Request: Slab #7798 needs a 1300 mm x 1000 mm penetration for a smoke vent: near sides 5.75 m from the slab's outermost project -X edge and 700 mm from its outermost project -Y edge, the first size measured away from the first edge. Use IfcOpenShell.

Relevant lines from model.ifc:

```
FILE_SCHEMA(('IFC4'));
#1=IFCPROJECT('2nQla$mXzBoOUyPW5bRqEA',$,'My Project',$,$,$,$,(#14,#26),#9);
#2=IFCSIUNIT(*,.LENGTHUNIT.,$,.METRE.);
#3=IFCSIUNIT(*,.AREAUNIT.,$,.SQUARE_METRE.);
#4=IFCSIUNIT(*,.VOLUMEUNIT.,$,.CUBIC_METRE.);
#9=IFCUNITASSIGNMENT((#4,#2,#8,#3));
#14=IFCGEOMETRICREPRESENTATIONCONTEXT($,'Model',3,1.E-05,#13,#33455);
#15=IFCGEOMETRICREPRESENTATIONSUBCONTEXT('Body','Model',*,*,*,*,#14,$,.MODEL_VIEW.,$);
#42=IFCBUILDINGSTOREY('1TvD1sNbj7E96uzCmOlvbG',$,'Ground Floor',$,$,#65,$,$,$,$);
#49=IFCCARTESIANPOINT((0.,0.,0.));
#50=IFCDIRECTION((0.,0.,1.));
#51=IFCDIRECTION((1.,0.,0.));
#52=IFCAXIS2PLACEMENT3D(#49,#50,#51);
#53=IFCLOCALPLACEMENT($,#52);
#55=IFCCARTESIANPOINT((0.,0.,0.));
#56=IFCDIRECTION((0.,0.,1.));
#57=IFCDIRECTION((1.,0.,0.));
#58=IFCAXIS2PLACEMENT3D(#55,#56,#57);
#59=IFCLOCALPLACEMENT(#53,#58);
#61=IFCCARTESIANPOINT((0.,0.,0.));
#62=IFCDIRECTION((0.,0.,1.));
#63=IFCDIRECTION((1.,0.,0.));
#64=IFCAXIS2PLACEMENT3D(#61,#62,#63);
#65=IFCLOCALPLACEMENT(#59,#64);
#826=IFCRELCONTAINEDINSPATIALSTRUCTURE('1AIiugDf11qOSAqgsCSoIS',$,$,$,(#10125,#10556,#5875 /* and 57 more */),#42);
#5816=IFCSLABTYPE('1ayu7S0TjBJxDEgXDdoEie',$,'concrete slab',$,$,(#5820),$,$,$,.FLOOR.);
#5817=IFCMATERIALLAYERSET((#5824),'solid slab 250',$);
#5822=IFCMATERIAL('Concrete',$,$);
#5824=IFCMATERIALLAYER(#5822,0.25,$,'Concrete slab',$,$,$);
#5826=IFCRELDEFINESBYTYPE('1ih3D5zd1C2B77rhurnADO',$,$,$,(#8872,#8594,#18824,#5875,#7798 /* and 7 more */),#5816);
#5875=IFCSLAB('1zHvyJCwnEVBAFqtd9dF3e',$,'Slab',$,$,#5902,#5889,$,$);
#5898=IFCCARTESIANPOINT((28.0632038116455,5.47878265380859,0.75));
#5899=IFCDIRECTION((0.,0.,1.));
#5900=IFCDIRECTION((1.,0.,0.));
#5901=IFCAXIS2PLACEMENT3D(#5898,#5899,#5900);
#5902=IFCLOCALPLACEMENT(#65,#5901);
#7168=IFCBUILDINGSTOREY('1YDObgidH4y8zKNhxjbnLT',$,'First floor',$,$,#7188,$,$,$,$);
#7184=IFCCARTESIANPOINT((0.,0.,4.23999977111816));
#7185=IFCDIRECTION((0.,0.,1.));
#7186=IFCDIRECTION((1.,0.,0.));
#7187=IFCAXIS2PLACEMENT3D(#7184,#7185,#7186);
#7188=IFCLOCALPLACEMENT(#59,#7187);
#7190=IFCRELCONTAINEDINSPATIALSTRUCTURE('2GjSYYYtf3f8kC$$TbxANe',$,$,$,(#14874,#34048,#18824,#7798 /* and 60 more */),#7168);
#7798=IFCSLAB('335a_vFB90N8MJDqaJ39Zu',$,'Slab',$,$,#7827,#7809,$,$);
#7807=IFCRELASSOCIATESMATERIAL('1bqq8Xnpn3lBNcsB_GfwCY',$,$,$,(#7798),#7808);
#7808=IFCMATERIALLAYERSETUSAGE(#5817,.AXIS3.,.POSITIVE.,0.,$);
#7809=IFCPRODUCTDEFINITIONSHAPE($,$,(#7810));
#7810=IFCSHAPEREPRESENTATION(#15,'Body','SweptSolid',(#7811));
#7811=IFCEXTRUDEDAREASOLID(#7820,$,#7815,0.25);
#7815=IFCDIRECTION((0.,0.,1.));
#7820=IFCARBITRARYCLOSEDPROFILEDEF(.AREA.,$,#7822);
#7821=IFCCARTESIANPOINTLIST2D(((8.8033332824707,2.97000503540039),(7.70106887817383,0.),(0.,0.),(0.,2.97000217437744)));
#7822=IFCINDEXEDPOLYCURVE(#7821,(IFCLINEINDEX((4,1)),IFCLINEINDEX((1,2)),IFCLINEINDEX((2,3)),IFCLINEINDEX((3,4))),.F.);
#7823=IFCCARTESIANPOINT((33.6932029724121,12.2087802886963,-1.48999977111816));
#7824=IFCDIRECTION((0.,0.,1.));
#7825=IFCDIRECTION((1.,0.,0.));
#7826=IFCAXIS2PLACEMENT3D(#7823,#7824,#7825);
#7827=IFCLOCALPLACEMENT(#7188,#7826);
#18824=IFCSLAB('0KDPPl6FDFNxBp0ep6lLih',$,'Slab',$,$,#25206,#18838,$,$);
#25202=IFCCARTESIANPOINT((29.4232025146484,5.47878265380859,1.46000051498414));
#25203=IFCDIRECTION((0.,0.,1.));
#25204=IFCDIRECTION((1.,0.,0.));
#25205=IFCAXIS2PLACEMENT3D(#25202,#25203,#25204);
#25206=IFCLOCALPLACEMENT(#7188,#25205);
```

```python
import numpy as np
import ifcopenshell
import ifcopenshell.api.feature
import ifcopenshell.api.geometry
import ifcopenshell.api.root
import ifcopenshell.geom
import ifcopenshell.util.placement
import ifcopenshell.util.representation
import ifcopenshell.util.shape
import ifcopenshell.util.unit

model = ifcopenshell.open("model.ifc")
unit_scale = ifcopenshell.util.unit.calculate_unit_scale(model)
settings = ifcopenshell.geom.settings()


def volume(element):
    """Net volume in cubic metres, openings subtracted."""
    shape = ifcopenshell.geom.create_shape(settings, element)
    return ifcopenshell.util.shape.get_volume(shape.geometry)


slab = model.by_guid("335a_vFB90N8MJDqaJ39Zu")
before = volume(slab)

# Extent in the slab's own axes, in metres. The edges named are its -X and -Y sides.
slab_shape = ifcopenshell.geom.create_shape(settings, slab)
vertices = ifcopenshell.util.shape.get_vertices(slab_shape.geometry)
x_min, y_min, bottom = vertices.min(axis=0)
top = vertices[:, 2].max()

opening = ifcopenshell.api.root.create_entity(model, ifc_class="IfcOpeningElement", name="Smoke vent opening", predefined_type="OPENING")
context = ifcopenshell.util.representation.get_context(model, "Model", "Body", "MODEL_VIEW")
width, depth = 1.3, 1
outline = [(0.0, 0.0), (width, 0.0), (width, depth), (0.0, depth), (0.0, 0.0)]
# Overshoot both faces by 50 mm so the cut is clean.
shape = ifcopenshell.api.geometry.add_slab_representation(
    model, context=context, depth=top - bottom + 0.1, polyline=outline
)
ifcopenshell.api.geometry.assign_representation(model, product=opening, representation=shape)

matrix = ifcopenshell.util.placement.get_local_placement(slab.ObjectPlacement)
matrix[:, 3] = matrix @ np.append(np.array([x_min + 5.75, y_min + 0.7, bottom - 0.05]) / unit_scale, 1.0)
ifcopenshell.api.geometry.edit_object_placement(model, product=opening, matrix=matrix, is_si=False)
ifcopenshell.api.feature.add_feature(model, feature=opening, element=slab)

after = volume(slab)

print(f"slab volume {before:.3f} -> {after:.3f} m3")

model.write("model_v2.ifc")
```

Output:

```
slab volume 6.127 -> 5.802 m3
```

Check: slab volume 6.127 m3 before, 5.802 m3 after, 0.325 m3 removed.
